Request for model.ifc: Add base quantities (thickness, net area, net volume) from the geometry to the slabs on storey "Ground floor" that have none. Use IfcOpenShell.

First a look at what the model holds.

```python
import ifcopenshell
import ifcopenshell.util.element
import ifcopenshell.util.unit

model = ifcopenshell.open("model.ifc")
print(model.schema)
for unit_type in ("LENGTHUNIT", "AREAUNIT", "VOLUMEUNIT"):
    print(unit_type, ifcopenshell.util.unit.calculate_unit_scale(model, unit_type))
storey = next(s for s in model.by_type("IfcBuildingStorey") if s.Name == "Ground floor")
slabs = [e for e in ifcopenshell.util.element.get_decomposition(storey) if e.is_a("IfcSlab")]
for e in sorted(slabs, key=lambda e: e.id()):
    print(e.id(), e.is_a(), e.Name, list(ifcopenshell.util.element.get_psets(e, qtos_only=True)), sep=" | ")
```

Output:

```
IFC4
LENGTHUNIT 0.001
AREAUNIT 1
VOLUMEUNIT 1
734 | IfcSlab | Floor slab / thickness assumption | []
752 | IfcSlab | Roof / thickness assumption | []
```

```python
import ifcopenshell
import ifcopenshell.api.pset
import ifcopenshell.geom
import ifcopenshell.util.element
import ifcopenshell.util.shape
import ifcopenshell.util.unit

model = ifcopenshell.open("model.ifc")
unit_scale = ifcopenshell.util.unit.calculate_unit_scale(model)
area_scale = ifcopenshell.util.unit.calculate_unit_scale(model, "AREAUNIT")
volume_scale = ifcopenshell.util.unit.calculate_unit_scale(model, "VOLUMEUNIT")
settings = ifcopenshell.geom.settings()

storey = next(s for s in model.by_type("IfcBuildingStorey") if s.Name == "Ground floor")
slabs = [e for e in ifcopenshell.util.element.get_decomposition(storey) if e.is_a("IfcSlab")]

for e in sorted(slabs, key=lambda e: e.id()):
    if ifcopenshell.util.element.get_psets(e, qtos_only=True, should_inherit=False):
        continue
    # Geometry comes back in metres, in the element's own axes.
    shape = ifcopenshell.geom.create_shape(settings, e)
    values = {
        "Width": ifcopenshell.util.shape.get_z(shape.geometry) / unit_scale,
        "NetArea": ifcopenshell.util.shape.get_footprint_area(shape.geometry) / area_scale,
        "NetVolume": ifcopenshell.util.shape.get_volume(shape.geometry) / volume_scale,
    }
    qto = ifcopenshell.api.pset.add_qto(model, product=e, name="Qto_SlabBaseQuantities")
    ifcopenshell.api.pset.edit_qto(model, qto=qto, properties=values)
    print(e.id(), {k: round(v, 3) for k, v in values.items()})

model.write("model_rev.ifc")
```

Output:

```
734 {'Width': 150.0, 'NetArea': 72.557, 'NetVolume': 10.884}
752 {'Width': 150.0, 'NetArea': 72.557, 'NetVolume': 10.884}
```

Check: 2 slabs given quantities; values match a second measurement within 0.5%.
